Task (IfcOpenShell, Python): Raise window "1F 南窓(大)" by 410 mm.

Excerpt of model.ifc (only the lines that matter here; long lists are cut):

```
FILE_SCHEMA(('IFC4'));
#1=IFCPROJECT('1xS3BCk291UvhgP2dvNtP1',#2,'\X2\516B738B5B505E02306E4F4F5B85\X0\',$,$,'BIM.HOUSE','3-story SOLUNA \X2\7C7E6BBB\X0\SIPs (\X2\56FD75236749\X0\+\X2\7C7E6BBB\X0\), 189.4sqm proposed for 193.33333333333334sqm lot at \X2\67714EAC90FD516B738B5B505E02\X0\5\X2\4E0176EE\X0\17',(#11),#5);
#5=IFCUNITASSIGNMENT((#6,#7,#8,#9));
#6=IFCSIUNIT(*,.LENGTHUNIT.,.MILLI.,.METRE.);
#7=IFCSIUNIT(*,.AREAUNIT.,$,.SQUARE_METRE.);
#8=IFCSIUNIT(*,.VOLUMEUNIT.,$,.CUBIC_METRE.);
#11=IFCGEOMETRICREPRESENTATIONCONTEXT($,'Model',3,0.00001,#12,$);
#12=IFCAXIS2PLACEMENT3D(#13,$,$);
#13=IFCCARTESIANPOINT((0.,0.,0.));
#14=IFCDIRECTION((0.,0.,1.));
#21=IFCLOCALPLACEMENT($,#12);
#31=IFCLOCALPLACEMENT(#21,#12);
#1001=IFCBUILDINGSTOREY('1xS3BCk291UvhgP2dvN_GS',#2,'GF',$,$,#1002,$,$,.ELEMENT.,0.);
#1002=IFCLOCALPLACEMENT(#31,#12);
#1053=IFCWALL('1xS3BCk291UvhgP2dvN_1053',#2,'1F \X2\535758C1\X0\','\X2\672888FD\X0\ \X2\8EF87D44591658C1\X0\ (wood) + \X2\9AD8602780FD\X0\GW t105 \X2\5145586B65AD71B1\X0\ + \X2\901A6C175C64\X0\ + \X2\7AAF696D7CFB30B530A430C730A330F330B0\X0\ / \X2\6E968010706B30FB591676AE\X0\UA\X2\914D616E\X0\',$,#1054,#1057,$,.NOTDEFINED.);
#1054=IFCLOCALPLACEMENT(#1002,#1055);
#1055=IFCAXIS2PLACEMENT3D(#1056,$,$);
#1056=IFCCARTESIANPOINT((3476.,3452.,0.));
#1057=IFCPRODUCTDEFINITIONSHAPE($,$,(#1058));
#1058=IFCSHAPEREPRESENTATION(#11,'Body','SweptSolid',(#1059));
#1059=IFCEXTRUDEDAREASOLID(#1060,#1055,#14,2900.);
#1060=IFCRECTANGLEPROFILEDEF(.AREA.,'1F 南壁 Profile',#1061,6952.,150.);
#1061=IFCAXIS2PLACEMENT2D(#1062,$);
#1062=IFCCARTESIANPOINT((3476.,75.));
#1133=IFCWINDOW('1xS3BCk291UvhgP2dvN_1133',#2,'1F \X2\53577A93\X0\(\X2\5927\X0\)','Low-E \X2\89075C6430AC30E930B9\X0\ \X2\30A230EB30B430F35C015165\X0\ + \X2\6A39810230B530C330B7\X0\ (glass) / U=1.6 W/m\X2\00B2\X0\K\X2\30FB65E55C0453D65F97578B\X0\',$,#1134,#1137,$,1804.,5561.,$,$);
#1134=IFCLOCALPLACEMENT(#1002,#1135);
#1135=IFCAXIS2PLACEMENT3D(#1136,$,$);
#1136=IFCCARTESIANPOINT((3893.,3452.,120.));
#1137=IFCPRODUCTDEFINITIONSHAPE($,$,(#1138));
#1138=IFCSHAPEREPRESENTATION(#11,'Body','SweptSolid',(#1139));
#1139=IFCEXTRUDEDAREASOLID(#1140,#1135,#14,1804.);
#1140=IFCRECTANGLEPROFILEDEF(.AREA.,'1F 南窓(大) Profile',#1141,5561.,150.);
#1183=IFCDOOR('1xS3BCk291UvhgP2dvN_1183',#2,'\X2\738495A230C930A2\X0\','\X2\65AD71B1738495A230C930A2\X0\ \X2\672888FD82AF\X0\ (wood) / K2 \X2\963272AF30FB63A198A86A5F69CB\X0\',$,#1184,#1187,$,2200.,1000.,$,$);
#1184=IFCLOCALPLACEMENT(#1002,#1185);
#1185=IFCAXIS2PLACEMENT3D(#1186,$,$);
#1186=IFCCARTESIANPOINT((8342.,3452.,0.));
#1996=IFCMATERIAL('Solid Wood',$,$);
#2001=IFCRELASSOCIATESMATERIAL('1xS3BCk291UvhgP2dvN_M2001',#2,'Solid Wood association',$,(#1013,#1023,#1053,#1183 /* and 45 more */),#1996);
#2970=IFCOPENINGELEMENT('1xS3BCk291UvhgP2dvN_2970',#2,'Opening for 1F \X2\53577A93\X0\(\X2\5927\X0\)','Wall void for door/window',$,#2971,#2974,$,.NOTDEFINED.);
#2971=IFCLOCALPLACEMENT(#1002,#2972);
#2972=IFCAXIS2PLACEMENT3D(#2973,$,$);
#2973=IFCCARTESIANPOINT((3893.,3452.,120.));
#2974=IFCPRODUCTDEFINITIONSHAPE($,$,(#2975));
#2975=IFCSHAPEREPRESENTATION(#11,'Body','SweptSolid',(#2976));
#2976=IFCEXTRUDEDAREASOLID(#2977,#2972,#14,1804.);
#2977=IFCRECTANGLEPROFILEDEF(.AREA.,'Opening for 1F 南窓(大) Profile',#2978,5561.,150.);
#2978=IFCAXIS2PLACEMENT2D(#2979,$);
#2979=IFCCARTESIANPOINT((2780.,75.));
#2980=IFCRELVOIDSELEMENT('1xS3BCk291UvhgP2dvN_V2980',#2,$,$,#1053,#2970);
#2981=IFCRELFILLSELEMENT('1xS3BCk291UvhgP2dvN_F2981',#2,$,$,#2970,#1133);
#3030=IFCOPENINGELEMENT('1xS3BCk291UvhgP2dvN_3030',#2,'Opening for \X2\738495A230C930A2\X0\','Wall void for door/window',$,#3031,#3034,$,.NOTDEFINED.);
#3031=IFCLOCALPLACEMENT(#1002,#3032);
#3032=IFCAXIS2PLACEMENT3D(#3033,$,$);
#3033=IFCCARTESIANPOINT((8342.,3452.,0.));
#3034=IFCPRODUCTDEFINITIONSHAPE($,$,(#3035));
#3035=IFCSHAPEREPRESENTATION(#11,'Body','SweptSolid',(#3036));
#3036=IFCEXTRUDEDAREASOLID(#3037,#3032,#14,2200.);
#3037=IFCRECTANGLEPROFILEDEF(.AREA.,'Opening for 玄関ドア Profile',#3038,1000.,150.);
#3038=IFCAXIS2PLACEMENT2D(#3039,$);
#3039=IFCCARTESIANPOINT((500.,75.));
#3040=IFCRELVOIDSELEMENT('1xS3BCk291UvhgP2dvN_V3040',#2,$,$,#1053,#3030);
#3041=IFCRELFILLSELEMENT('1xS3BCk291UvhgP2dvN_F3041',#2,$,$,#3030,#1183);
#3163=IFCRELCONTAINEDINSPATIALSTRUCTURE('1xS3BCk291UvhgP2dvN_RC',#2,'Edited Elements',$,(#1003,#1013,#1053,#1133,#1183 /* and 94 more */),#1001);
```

```python
import numpy as np
import ifcopenshell
import ifcopenshell.api.geometry
import ifcopenshell.util.placement
import ifcopenshell.util.unit

model = ifcopenshell.open("model.ifc")
unit_scale = ifcopenshell.util.unit.calculate_unit_scale(model)

window = model.by_guid("1xS3BCk291UvhgP2dvN_1133")
opening = window.FillsVoids[0].RelatingOpeningElement
dz = 410.0

shift = np.array([0.0, 0.0, dz])
# The window is not placed relative to its opening, so move both.
for product in (opening, window):
    matrix = ifcopenshell.util.placement.get_local_placement(product.ObjectPlacement)
    matrix[:3, 3] += shift
    ifcopenshell.api.geometry.edit_object_placement(model, product=product, matrix=matrix, is_si=False)

print(f"moved by {dz * unit_scale:+.3f} m")

model.write("model_rev.ifc")
```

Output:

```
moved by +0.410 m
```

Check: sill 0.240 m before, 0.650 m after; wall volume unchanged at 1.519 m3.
